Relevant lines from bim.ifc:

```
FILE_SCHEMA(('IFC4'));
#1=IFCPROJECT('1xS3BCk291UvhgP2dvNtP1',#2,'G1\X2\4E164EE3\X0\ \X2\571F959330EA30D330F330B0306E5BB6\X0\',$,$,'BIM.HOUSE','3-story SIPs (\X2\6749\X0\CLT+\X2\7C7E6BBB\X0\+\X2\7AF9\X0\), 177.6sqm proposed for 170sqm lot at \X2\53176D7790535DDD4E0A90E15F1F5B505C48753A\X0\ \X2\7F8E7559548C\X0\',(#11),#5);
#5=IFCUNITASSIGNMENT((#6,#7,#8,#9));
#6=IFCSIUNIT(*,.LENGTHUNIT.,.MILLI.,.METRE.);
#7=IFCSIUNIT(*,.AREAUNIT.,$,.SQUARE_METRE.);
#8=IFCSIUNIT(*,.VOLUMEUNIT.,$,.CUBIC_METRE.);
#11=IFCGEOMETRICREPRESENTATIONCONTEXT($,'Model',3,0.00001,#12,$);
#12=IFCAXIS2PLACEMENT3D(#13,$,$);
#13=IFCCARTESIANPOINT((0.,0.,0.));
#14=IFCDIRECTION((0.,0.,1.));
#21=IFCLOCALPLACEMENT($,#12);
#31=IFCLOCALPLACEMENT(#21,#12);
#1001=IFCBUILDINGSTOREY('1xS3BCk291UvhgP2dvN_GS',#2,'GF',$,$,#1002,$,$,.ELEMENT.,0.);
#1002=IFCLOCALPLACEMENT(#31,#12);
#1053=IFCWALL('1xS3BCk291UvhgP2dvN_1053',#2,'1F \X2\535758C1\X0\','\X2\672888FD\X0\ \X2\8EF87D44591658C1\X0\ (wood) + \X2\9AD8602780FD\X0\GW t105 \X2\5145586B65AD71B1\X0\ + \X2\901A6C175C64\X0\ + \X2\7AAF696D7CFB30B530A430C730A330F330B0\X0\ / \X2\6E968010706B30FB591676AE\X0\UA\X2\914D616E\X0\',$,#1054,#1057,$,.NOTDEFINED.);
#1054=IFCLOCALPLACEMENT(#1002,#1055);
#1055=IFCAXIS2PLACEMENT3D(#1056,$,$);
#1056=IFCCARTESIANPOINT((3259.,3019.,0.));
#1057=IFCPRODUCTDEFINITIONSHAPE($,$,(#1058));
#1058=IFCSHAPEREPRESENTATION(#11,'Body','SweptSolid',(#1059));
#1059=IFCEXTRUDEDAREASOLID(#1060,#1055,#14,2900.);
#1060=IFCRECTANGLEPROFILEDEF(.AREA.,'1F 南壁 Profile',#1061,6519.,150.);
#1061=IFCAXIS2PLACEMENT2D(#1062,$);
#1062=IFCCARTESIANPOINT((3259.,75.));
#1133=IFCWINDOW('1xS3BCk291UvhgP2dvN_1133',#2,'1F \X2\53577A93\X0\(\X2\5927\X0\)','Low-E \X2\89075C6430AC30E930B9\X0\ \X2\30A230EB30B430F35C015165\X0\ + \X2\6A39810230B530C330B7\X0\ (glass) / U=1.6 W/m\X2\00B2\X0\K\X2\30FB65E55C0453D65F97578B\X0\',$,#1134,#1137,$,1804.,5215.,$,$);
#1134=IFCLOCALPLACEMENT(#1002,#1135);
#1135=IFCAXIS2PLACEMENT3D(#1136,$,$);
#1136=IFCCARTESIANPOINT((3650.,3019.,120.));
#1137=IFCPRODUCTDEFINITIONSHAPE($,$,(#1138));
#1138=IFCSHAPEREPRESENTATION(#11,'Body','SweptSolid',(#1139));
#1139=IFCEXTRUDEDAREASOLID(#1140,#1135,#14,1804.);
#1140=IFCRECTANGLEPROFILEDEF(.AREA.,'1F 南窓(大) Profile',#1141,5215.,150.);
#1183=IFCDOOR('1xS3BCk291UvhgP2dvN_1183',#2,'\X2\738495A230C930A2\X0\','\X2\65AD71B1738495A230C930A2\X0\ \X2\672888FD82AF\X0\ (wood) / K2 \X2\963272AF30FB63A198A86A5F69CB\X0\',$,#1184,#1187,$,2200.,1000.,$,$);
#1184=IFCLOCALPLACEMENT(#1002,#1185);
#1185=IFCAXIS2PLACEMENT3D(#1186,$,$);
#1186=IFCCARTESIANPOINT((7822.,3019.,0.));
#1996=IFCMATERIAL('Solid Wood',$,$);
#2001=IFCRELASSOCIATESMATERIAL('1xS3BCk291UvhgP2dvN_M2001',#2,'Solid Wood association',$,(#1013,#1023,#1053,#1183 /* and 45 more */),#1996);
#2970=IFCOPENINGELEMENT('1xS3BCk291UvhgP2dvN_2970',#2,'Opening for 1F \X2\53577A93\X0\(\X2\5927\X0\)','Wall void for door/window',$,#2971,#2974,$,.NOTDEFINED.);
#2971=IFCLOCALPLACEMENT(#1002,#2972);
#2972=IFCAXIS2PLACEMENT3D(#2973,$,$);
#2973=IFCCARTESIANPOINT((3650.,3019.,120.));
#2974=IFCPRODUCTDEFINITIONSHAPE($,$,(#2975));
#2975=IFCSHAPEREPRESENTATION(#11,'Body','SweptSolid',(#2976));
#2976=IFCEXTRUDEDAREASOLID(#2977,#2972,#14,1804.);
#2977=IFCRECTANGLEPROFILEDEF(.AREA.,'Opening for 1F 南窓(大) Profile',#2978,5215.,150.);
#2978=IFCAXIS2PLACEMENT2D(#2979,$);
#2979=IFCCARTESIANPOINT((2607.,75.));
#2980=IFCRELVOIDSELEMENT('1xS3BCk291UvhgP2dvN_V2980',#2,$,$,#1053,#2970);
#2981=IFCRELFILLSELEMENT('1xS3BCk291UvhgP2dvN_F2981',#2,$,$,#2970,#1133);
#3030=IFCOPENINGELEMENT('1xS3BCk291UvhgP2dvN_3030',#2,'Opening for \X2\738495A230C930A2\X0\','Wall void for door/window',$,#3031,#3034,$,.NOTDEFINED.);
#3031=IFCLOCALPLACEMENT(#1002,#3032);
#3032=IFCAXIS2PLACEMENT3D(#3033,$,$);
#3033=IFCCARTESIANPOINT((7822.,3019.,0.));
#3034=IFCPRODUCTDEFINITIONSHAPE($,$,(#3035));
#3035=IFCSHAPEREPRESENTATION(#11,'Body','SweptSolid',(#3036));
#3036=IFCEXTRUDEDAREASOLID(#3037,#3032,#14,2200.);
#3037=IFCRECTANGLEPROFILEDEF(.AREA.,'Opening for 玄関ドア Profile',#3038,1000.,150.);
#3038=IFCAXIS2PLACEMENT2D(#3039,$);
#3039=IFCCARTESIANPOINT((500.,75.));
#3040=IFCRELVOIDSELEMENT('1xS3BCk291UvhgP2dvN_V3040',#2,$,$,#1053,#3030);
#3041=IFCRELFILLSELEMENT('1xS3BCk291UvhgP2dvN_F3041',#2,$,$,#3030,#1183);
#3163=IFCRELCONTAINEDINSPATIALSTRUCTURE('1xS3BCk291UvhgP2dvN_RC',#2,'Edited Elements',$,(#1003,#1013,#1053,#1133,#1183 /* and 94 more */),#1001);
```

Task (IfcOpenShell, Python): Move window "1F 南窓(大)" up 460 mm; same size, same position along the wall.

```python
import numpy as np
import ifcopenshell
import ifcopenshell.api.geometry
import ifcopenshell.util.placement
import ifcopenshell.util.unit

model = ifcopenshell.open("bim.ifc")
unit_scale = ifcopenshell.util.unit.calculate_unit_scale(model)

window = model.by_guid("1xS3BCk291UvhgP2dvN_1133")
opening = window.FillsVoids[0].RelatingOpeningElement
dz = 460.0

shift = np.array([0.0, 0.0, dz])
# The window is not placed relative to its opening, so move both.
for product in (opening, window):
    matrix = ifcopenshell.util.placement.get_local_placement(product.ObjectPlacement)
    matrix[:3, 3] += shift
    ifcopenshell.api.geometry.edit_object_placement(model, product=product, matrix=matrix, is_si=False)

print(f"moved by {dz * unit_scale:+.3f} m")

model.write("bim-out.ifc")
```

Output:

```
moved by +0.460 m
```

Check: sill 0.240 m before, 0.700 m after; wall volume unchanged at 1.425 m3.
